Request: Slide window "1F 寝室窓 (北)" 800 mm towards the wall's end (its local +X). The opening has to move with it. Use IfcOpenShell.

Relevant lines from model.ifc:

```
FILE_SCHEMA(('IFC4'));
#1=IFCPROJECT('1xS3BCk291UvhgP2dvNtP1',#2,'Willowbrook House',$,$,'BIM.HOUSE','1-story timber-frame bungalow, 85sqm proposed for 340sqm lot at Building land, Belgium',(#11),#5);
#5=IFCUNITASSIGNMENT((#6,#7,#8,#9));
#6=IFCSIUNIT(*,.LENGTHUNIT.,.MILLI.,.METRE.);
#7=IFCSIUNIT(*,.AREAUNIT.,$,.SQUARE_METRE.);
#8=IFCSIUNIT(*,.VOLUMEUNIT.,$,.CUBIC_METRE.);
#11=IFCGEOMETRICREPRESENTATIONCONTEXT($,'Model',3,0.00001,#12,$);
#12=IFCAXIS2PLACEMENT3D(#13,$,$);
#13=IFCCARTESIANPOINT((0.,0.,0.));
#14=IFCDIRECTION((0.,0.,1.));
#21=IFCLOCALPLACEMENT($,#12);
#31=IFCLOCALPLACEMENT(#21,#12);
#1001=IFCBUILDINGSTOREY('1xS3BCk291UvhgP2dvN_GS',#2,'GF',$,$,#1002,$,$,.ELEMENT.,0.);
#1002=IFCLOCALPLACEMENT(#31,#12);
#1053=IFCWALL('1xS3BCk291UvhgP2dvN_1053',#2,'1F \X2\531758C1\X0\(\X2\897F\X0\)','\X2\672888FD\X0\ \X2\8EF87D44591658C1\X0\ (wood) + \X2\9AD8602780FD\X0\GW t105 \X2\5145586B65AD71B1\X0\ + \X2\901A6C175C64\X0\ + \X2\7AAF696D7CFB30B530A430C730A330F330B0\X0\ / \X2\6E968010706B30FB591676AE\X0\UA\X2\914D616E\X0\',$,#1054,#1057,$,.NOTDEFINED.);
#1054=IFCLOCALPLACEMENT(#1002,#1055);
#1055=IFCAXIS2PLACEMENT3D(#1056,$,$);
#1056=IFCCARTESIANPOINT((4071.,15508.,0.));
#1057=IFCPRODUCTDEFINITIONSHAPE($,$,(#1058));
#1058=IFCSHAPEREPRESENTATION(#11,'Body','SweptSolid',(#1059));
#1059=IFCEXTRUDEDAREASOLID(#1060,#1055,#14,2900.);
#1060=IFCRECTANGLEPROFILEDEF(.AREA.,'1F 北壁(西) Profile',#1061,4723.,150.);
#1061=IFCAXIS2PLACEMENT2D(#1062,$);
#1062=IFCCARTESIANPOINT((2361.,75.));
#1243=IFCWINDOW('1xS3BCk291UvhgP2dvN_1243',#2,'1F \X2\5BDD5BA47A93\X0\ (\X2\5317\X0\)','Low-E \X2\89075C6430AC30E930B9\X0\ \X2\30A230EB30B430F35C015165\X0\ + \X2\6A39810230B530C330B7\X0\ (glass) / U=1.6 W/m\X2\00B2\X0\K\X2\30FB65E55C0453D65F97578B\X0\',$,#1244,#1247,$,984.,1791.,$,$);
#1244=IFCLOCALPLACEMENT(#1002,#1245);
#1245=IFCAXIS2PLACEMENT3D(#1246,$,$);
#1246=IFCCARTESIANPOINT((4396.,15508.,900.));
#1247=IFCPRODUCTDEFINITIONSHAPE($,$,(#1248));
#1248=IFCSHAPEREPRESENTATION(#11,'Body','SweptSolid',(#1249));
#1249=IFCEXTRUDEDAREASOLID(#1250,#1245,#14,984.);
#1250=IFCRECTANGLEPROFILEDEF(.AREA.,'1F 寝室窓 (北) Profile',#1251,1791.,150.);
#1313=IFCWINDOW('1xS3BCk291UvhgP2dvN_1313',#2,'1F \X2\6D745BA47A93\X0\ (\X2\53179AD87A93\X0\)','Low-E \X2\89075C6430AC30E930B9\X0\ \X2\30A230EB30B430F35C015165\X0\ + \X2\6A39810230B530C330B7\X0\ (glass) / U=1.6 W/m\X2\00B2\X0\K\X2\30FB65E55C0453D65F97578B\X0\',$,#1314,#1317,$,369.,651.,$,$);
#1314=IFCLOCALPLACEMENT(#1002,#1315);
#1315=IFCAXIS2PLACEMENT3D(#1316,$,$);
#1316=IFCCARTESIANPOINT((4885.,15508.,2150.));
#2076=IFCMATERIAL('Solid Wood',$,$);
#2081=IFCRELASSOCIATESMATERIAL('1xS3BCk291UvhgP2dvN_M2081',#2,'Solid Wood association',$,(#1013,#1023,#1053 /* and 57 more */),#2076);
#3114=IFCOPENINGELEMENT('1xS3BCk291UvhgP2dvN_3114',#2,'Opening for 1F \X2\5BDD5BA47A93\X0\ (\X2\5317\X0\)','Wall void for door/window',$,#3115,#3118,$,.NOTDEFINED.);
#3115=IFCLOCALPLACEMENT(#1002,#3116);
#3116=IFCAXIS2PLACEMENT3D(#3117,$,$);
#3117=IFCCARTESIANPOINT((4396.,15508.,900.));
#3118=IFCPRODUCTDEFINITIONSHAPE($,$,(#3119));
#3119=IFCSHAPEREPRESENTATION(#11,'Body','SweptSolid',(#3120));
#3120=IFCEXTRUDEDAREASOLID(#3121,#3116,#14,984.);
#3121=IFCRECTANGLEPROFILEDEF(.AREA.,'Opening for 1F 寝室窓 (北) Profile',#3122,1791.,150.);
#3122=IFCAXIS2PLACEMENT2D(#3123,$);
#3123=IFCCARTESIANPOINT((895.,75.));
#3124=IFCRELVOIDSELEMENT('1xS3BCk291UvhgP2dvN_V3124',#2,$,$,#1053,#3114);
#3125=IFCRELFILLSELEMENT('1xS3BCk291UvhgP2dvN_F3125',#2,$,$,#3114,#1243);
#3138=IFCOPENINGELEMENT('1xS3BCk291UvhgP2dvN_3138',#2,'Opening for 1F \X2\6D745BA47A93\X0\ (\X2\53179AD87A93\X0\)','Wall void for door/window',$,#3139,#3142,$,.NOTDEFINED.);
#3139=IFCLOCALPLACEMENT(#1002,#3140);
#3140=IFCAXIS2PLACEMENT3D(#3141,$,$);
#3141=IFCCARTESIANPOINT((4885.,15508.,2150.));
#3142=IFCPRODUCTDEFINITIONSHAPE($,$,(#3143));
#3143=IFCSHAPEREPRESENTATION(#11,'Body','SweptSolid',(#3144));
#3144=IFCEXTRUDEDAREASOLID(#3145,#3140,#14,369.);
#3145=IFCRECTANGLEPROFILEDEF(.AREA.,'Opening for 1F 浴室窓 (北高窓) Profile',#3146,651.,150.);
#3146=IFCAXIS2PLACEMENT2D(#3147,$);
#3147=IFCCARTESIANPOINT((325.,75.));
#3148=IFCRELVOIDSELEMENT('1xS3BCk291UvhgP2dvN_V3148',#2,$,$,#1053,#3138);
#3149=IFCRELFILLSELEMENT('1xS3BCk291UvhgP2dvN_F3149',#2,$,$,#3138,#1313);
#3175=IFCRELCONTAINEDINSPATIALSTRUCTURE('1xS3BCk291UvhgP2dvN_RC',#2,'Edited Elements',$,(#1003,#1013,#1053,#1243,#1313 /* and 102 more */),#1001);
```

```python
import ifcopenshell
import ifcopenshell.api.geometry
import ifcopenshell.util.placement

model = ifcopenshell.open("model.ifc")

window = model.by_guid("1xS3BCk291UvhgP2dvN_1243")
opening = window.FillsVoids[0].RelatingOpeningElement
wall = opening.VoidsElements[0].RelatingBuildingElement

wall_matrix = ifcopenshell.util.placement.get_local_placement(wall.ObjectPlacement)
shift = wall_matrix[:3, 0] * 800.0
before = ifcopenshell.util.placement.get_local_placement(window.ObjectPlacement)[:3, 3].copy()

# The window is not placed relative to its opening, so move both.
for product in (opening, window):
    matrix = ifcopenshell.util.placement.get_local_placement(product.ObjectPlacement)
    matrix[:3, 3] += shift
    ifcopenshell.api.geometry.edit_object_placement(model, product=product, matrix=matrix, is_si=False)

after = ifcopenshell.util.placement.get_local_placement(window.ObjectPlacement)[:3, 3]
print("window moved by", (after - before).round(3) + 0.0)

model.write("model_edited.ifc")
```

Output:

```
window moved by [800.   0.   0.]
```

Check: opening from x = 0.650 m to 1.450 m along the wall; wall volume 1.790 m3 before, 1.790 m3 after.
